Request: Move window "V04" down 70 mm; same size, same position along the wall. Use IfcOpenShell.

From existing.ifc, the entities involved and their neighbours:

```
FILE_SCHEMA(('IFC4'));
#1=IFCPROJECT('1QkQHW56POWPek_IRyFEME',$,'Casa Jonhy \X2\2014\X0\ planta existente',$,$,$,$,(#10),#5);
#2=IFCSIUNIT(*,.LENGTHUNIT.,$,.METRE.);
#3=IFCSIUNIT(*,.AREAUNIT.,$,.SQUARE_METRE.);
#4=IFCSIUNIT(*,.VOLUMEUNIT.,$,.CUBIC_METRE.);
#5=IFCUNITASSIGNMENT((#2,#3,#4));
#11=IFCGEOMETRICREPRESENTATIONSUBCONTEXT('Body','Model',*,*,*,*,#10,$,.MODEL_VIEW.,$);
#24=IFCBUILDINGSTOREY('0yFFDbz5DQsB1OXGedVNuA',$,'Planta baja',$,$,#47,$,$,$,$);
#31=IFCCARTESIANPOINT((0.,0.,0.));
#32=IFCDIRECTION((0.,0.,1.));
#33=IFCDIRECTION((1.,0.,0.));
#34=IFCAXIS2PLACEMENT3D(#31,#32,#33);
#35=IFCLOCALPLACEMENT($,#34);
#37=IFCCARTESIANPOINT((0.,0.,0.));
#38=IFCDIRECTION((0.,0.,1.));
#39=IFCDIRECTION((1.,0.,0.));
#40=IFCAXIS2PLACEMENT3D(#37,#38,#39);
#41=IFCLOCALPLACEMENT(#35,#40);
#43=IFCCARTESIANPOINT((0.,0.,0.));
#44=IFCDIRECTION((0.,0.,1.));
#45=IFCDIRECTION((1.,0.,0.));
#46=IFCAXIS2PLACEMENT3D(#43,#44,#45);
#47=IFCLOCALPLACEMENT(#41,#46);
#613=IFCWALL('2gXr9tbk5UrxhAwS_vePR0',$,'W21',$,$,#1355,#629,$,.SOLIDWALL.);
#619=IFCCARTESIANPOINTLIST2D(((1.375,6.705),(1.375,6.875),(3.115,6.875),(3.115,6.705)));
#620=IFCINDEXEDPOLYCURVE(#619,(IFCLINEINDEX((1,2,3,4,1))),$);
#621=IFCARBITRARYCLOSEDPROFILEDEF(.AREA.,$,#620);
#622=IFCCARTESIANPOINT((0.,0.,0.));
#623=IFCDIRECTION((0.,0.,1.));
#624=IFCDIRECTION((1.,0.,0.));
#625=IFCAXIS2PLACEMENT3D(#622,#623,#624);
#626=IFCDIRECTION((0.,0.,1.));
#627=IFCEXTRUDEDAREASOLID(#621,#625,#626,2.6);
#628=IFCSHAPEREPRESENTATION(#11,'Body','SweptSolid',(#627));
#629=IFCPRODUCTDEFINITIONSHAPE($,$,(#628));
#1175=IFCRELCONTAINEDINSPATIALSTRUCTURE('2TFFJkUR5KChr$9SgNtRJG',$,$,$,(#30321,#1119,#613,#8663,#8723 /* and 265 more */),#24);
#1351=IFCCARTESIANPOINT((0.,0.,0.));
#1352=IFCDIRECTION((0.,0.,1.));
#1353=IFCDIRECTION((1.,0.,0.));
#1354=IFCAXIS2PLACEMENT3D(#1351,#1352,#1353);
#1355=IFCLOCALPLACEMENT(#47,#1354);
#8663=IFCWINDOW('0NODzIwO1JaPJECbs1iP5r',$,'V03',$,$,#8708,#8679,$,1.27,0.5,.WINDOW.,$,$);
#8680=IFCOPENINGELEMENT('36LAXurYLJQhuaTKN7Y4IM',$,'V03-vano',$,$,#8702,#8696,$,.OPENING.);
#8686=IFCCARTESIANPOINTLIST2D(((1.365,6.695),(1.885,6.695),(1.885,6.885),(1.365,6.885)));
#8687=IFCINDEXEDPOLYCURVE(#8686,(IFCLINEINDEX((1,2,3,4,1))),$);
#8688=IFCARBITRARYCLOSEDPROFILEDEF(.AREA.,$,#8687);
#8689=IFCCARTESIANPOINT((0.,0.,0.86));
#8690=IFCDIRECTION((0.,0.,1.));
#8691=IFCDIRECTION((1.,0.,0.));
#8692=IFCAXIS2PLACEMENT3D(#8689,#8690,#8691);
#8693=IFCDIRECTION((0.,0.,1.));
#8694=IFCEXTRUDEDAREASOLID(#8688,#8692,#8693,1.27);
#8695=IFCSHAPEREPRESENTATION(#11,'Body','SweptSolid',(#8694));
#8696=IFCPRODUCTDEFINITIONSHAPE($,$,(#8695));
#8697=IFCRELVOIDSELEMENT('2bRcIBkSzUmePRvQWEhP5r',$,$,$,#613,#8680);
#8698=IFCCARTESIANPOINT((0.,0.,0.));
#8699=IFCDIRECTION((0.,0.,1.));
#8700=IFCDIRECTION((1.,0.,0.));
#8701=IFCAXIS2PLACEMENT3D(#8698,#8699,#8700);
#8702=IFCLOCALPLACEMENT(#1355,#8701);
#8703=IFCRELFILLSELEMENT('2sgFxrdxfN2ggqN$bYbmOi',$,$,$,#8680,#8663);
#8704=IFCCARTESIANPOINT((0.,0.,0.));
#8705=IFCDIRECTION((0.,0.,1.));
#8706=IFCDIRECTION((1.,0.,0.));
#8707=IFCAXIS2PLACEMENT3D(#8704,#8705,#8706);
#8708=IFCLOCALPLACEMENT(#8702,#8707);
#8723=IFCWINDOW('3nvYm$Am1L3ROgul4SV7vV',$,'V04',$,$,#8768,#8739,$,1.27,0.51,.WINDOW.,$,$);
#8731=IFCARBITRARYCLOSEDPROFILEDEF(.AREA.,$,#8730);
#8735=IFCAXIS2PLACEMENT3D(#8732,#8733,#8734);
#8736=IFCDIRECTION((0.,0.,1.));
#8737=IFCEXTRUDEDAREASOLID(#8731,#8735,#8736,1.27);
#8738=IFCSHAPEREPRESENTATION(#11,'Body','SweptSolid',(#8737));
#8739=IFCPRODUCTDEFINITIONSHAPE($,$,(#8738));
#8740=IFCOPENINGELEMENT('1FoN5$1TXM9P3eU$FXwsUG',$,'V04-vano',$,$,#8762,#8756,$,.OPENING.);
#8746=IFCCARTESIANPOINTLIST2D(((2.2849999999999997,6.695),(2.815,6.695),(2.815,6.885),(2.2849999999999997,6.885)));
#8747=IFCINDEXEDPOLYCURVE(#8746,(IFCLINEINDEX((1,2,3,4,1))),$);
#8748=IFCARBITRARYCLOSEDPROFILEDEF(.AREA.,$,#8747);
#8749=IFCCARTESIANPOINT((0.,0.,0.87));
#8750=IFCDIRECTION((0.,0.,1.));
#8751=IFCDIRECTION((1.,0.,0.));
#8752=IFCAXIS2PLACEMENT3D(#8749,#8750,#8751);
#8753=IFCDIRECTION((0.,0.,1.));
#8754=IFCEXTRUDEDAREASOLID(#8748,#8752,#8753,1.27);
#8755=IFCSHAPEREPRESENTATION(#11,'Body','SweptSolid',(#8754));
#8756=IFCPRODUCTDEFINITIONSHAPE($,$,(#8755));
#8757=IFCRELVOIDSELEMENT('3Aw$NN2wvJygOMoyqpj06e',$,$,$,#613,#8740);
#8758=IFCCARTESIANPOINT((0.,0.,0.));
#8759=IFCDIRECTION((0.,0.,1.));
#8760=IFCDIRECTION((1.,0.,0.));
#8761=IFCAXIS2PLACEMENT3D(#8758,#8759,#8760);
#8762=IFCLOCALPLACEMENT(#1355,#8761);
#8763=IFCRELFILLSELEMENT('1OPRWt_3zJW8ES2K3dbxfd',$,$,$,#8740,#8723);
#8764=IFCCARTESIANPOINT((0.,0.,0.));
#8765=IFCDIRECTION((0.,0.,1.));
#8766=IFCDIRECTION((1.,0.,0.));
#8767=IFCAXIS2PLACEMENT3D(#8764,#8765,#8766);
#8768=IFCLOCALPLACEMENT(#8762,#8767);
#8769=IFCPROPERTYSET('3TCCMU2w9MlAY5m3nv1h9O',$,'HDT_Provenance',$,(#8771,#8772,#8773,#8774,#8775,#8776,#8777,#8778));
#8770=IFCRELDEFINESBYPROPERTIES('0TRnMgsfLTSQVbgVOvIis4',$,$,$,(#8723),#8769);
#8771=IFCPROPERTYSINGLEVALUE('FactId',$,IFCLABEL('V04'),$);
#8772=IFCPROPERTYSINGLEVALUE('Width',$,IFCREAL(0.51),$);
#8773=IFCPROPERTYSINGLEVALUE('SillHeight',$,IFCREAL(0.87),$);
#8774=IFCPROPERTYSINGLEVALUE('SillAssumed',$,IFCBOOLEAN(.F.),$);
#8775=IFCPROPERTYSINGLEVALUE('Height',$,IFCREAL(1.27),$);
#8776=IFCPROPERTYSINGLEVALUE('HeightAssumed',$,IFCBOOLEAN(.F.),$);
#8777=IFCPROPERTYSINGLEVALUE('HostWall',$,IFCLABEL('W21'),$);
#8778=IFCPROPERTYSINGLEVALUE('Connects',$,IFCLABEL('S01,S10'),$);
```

```python
import numpy as np
import ifcopenshell
import ifcopenshell.api.geometry
import ifcopenshell.api.pset
import ifcopenshell.util.element
import ifcopenshell.util.placement
import ifcopenshell.util.unit

model = ifcopenshell.open("existing.ifc")
unit_scale = ifcopenshell.util.unit.calculate_unit_scale(model)

window = model.by_guid("3nvYm$Am1L3ROgul4SV7vV")
opening = window.FillsVoids[0].RelatingOpeningElement
dz = -0.07 / unit_scale

shift = np.array([0.0, 0.0, dz])
# The window is placed relative to its opening, so it follows when the opening moves.
matrix = ifcopenshell.util.placement.get_local_placement(opening.ObjectPlacement)
matrix[:3, 3] += shift
ifcopenshell.api.geometry.edit_object_placement(
    model, product=opening, matrix=matrix, is_si=False, should_transform_children=True
)

# Keep the stored heights in step.
pset = model.by_id(ifcopenshell.util.element.get_pset(window, "HDT_Provenance", should_inherit=False)["id"])
ifcopenshell.api.pset.edit_pset(model, pset=pset, properties={
    "SillHeight": model.create_entity("IfcReal", ifcopenshell.util.element.get_pset(window, "HDT_Provenance", "SillHeight") + dz),
})

print(f"moved by {dz * unit_scale:+.3f} m")

model.write("existing-out.ifc")
```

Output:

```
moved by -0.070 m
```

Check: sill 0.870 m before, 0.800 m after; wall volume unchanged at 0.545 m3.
